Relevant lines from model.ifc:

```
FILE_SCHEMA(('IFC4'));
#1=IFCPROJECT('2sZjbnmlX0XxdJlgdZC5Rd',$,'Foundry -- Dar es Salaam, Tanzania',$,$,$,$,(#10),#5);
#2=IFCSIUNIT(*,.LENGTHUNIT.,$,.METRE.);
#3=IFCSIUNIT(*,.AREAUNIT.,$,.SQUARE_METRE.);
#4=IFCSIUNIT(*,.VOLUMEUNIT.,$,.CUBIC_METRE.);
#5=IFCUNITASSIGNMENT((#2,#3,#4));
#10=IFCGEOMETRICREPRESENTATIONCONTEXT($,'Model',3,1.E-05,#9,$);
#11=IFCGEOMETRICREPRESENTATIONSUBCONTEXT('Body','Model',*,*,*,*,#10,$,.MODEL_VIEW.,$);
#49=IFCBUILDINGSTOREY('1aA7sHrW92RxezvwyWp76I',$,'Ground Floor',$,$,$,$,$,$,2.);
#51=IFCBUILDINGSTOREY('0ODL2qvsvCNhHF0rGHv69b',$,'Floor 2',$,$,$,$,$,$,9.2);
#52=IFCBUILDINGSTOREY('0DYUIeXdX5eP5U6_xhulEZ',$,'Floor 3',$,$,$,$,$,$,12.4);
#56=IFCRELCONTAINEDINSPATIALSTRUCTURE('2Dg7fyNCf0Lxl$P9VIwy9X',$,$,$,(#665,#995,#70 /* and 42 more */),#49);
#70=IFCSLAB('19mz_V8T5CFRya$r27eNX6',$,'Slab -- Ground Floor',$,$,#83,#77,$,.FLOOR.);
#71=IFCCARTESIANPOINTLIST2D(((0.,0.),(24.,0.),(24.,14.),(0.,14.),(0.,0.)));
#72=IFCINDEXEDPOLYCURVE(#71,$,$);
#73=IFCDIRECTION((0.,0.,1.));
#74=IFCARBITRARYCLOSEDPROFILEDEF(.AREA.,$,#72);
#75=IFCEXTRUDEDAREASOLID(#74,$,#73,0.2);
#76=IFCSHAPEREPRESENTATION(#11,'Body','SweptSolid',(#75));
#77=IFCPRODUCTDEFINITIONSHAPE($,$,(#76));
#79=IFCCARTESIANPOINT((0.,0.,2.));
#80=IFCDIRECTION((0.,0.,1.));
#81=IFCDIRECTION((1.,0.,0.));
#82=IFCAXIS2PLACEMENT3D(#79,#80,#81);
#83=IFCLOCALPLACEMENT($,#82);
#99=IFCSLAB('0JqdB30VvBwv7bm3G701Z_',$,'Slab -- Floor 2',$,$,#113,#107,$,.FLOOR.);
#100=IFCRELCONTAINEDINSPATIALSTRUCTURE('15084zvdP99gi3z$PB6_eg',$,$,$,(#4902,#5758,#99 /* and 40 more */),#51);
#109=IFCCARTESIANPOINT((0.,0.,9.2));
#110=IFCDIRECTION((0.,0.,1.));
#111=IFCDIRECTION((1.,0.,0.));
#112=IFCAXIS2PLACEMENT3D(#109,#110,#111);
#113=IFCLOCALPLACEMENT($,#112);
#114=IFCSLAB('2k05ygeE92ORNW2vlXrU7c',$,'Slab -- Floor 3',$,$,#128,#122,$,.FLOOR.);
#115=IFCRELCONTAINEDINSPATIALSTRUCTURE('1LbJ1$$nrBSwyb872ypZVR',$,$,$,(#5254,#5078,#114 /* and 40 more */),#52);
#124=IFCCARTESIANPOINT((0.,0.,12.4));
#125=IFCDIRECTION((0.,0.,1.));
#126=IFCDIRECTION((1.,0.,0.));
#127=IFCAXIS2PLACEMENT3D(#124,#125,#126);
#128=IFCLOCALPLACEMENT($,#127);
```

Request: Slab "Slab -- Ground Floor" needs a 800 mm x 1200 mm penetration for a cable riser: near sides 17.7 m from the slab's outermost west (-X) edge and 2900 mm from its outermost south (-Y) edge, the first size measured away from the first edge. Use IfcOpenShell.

```python
import numpy as np
import ifcopenshell
import ifcopenshell.api.feature
import ifcopenshell.api.geometry
import ifcopenshell.api.root
import ifcopenshell.geom
import ifcopenshell.util.placement
import ifcopenshell.util.representation
import ifcopenshell.util.shape
import ifcopenshell.util.unit

model = ifcopenshell.open("model.ifc")
unit_scale = ifcopenshell.util.unit.calculate_unit_scale(model)
settings = ifcopenshell.geom.settings()


def volume(element):
    """Net volume in cubic metres, openings subtracted."""
    shape = ifcopenshell.geom.create_shape(settings, element)
    return ifcopenshell.util.shape.get_volume(shape.geometry)


slab = model.by_id(70)
before = volume(slab)

# Extent in the slab's own axes, in metres. The edges named are its -X and -Y sides.
slab_shape = ifcopenshell.geom.create_shape(settings, slab)
vertices = ifcopenshell.util.shape.get_vertices(slab_shape.geometry)
x_min, y_min, bottom = vertices.min(axis=0)
top = vertices[:, 2].max()

opening = ifcopenshell.api.root.create_entity(model, ifc_class="IfcOpeningElement", name="Cable riser opening", predefined_type="OPENING")
context = ifcopenshell.util.representation.get_context(model, "Model", "Body", "MODEL_VIEW")
width, depth = 0.8, 1.2
outline = [(0.0, 0.0), (width, 0.0), (width, depth), (0.0, depth), (0.0, 0.0)]
# Overshoot both faces by 50 mm so the cut is clean.
shape = ifcopenshell.api.geometry.add_slab_representation(
    model, context=context, depth=top - bottom + 0.1, polyline=outline
)
ifcopenshell.api.geometry.assign_representation(model, product=opening, representation=shape)

matrix = ifcopenshell.util.placement.get_local_placement(slab.ObjectPlacement)
matrix[:, 3] = matrix @ np.append(np.array([x_min + 17.7, y_min + 2.9, bottom - 0.05]) / unit_scale, 1.0)
ifcopenshell.api.geometry.edit_object_placement(model, product=opening, matrix=matrix, is_si=False)
ifcopenshell.api.feature.add_feature(model, feature=opening, element=slab)

after = volume(slab)

print(f"slab volume {before:.3f} -> {after:.3f} m3")

model.write("model_edited.ifc")
```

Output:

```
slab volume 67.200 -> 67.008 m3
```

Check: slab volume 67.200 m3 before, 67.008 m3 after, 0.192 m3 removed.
